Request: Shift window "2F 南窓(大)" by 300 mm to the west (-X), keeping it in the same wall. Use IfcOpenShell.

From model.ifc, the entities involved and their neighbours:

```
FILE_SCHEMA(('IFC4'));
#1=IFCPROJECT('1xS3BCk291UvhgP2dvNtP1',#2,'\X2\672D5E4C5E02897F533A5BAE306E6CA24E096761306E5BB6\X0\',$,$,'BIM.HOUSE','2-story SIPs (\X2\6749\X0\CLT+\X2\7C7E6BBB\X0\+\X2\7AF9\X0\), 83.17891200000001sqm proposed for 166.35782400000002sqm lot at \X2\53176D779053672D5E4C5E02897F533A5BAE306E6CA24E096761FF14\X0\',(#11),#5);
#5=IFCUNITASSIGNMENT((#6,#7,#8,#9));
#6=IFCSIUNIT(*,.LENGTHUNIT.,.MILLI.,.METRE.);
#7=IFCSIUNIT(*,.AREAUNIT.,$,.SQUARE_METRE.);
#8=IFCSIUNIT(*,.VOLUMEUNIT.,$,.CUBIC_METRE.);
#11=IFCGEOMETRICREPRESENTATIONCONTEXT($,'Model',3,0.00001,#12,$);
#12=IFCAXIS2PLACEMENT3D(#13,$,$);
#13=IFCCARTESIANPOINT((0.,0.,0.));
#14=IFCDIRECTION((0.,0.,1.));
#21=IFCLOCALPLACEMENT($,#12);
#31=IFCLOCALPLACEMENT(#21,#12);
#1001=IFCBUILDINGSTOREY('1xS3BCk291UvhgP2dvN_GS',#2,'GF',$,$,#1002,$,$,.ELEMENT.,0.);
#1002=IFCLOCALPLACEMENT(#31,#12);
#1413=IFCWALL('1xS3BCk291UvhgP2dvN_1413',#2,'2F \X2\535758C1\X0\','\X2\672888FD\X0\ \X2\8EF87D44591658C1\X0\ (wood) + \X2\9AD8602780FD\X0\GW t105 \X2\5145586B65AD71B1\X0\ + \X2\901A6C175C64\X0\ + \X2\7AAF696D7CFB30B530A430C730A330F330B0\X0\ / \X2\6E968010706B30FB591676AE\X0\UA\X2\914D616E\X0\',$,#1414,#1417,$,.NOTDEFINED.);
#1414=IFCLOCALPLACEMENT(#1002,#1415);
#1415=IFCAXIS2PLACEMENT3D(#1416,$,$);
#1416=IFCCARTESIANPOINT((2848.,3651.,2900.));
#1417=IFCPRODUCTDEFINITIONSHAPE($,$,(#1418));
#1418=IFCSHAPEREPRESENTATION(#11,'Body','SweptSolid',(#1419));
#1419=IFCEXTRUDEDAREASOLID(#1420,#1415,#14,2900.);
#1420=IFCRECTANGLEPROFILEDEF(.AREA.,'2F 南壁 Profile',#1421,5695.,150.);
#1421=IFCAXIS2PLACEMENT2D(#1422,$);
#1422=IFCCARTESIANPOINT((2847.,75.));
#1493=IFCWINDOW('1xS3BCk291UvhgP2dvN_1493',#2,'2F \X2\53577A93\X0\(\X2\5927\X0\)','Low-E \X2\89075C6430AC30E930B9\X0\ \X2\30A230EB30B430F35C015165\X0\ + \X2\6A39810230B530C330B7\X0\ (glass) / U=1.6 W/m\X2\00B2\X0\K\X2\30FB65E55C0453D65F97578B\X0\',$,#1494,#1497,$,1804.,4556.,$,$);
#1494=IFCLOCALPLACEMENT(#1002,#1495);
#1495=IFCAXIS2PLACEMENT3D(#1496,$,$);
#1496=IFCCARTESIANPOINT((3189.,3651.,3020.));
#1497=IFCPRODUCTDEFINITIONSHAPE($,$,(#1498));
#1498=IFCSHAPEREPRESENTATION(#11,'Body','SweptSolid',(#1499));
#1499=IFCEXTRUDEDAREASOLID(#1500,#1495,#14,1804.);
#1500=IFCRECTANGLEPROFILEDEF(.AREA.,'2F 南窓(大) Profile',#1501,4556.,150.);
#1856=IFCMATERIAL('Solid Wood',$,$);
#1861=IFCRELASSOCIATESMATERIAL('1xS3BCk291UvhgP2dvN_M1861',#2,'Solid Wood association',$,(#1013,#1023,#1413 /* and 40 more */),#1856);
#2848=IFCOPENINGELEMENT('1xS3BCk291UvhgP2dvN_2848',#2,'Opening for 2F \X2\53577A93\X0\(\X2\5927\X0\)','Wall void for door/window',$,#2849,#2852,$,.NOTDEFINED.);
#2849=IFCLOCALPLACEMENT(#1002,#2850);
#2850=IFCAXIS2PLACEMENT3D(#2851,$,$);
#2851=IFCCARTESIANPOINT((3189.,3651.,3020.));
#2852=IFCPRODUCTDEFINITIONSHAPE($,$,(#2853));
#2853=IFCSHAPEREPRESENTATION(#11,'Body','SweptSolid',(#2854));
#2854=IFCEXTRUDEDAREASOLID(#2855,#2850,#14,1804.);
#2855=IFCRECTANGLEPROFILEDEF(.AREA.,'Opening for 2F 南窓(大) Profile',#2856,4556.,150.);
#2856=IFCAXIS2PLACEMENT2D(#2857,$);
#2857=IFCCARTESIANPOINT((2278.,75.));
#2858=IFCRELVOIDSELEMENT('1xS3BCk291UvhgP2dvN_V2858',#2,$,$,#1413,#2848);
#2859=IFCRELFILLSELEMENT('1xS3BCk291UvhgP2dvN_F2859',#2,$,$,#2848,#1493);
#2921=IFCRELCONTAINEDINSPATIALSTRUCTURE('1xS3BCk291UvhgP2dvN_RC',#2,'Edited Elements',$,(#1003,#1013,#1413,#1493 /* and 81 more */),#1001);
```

```python
import ifcopenshell
import ifcopenshell.api.geometry
import ifcopenshell.util.placement
import ifcopenshell.util.unit

model = ifcopenshell.open("model.ifc")
unit_scale = ifcopenshell.util.unit.calculate_unit_scale(model)

window = model.by_id(1493)
opening = window.FillsVoids[0].RelatingOpeningElement
wall = opening.VoidsElements[0].RelatingBuildingElement

wall_matrix = ifcopenshell.util.placement.get_local_placement(wall.ObjectPlacement)
shift = wall_matrix[:3, 0] * -0.3 / unit_scale
before = ifcopenshell.util.placement.get_local_placement(window.ObjectPlacement)[:3, 3].copy()

# The window is not placed relative to its opening, so move both.
for product in (opening, window):
    matrix = ifcopenshell.util.placement.get_local_placement(product.ObjectPlacement)
    matrix[:3, 3] += shift
    ifcopenshell.api.geometry.edit_object_placement(model, product=product, matrix=matrix, is_si=False)

after = ifcopenshell.util.placement.get_local_placement(window.ObjectPlacement)[:3, 3]
print("window moved by", (after - before).round(3) + 0.0)

model.write("model_updated.ifc")
```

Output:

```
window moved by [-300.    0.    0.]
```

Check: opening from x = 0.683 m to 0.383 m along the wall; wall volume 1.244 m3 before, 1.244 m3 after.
